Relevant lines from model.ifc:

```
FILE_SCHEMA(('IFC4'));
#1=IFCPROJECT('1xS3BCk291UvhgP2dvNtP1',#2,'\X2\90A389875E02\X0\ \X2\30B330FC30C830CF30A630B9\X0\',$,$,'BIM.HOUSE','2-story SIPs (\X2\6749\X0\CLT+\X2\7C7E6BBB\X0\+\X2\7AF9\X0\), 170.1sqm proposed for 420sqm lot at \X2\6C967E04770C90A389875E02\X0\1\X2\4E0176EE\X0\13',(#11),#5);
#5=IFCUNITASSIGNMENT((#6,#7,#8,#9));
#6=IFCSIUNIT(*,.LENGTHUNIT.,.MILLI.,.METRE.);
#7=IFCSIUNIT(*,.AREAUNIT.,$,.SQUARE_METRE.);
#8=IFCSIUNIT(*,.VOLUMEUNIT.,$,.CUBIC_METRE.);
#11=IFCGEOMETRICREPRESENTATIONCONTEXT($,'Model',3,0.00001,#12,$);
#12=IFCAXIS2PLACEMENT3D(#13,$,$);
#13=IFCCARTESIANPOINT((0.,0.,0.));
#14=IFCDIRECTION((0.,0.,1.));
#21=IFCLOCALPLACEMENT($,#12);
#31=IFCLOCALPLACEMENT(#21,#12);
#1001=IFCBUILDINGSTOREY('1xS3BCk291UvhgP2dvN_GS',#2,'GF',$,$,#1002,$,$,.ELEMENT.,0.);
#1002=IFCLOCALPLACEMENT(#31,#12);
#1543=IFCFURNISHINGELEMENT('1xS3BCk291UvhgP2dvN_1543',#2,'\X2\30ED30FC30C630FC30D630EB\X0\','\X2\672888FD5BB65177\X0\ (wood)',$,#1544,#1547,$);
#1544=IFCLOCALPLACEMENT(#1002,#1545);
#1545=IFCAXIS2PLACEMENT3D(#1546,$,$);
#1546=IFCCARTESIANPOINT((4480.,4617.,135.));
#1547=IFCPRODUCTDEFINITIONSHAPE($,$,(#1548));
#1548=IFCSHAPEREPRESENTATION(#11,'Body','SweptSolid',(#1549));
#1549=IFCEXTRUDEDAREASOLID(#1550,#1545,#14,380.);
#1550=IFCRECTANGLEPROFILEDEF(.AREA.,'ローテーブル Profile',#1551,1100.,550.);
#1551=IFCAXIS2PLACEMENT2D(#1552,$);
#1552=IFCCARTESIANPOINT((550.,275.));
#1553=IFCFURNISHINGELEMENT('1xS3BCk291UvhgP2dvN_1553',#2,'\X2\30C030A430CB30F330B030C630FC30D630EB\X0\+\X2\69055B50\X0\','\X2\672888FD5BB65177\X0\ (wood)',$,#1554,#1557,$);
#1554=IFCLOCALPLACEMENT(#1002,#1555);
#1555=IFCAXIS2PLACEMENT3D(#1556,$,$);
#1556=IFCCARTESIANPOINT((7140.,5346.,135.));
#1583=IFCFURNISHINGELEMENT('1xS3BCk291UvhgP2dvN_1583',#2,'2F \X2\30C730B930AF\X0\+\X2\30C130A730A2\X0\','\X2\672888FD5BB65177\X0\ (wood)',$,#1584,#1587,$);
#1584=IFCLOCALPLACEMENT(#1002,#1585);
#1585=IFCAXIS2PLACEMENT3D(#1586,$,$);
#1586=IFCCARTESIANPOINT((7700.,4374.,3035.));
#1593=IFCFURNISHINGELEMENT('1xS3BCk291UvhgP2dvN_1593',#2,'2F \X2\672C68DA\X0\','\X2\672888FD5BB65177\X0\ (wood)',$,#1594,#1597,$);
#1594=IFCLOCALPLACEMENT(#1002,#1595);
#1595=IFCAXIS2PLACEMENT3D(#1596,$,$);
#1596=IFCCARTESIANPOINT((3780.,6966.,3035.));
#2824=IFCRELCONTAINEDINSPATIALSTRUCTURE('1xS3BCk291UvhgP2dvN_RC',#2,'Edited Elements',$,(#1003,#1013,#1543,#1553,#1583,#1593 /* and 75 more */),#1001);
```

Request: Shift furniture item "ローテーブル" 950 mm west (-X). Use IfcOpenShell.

```python
import ifcopenshell
import ifcopenshell.api.geometry
import ifcopenshell.util.placement
import ifcopenshell.util.unit

model = ifcopenshell.open("model.ifc")
unit_scale = ifcopenshell.util.unit.calculate_unit_scale(model)

item = model.by_guid("1xS3BCk291UvhgP2dvN_1543")
matrix = ifcopenshell.util.placement.get_local_placement(item.ObjectPlacement)
matrix[0, 3] -= 0.95 / unit_scale
ifcopenshell.api.geometry.edit_object_placement(model, product=item, matrix=matrix, is_si=False)

print(ifcopenshell.util.placement.get_local_placement(item.ObjectPlacement).round(3) + 0.0)

model.write("model_rev.ifc")
```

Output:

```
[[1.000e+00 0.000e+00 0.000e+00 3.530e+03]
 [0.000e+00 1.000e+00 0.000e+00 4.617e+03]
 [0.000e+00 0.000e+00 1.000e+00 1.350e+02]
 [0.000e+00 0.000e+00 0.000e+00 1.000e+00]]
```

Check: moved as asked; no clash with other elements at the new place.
